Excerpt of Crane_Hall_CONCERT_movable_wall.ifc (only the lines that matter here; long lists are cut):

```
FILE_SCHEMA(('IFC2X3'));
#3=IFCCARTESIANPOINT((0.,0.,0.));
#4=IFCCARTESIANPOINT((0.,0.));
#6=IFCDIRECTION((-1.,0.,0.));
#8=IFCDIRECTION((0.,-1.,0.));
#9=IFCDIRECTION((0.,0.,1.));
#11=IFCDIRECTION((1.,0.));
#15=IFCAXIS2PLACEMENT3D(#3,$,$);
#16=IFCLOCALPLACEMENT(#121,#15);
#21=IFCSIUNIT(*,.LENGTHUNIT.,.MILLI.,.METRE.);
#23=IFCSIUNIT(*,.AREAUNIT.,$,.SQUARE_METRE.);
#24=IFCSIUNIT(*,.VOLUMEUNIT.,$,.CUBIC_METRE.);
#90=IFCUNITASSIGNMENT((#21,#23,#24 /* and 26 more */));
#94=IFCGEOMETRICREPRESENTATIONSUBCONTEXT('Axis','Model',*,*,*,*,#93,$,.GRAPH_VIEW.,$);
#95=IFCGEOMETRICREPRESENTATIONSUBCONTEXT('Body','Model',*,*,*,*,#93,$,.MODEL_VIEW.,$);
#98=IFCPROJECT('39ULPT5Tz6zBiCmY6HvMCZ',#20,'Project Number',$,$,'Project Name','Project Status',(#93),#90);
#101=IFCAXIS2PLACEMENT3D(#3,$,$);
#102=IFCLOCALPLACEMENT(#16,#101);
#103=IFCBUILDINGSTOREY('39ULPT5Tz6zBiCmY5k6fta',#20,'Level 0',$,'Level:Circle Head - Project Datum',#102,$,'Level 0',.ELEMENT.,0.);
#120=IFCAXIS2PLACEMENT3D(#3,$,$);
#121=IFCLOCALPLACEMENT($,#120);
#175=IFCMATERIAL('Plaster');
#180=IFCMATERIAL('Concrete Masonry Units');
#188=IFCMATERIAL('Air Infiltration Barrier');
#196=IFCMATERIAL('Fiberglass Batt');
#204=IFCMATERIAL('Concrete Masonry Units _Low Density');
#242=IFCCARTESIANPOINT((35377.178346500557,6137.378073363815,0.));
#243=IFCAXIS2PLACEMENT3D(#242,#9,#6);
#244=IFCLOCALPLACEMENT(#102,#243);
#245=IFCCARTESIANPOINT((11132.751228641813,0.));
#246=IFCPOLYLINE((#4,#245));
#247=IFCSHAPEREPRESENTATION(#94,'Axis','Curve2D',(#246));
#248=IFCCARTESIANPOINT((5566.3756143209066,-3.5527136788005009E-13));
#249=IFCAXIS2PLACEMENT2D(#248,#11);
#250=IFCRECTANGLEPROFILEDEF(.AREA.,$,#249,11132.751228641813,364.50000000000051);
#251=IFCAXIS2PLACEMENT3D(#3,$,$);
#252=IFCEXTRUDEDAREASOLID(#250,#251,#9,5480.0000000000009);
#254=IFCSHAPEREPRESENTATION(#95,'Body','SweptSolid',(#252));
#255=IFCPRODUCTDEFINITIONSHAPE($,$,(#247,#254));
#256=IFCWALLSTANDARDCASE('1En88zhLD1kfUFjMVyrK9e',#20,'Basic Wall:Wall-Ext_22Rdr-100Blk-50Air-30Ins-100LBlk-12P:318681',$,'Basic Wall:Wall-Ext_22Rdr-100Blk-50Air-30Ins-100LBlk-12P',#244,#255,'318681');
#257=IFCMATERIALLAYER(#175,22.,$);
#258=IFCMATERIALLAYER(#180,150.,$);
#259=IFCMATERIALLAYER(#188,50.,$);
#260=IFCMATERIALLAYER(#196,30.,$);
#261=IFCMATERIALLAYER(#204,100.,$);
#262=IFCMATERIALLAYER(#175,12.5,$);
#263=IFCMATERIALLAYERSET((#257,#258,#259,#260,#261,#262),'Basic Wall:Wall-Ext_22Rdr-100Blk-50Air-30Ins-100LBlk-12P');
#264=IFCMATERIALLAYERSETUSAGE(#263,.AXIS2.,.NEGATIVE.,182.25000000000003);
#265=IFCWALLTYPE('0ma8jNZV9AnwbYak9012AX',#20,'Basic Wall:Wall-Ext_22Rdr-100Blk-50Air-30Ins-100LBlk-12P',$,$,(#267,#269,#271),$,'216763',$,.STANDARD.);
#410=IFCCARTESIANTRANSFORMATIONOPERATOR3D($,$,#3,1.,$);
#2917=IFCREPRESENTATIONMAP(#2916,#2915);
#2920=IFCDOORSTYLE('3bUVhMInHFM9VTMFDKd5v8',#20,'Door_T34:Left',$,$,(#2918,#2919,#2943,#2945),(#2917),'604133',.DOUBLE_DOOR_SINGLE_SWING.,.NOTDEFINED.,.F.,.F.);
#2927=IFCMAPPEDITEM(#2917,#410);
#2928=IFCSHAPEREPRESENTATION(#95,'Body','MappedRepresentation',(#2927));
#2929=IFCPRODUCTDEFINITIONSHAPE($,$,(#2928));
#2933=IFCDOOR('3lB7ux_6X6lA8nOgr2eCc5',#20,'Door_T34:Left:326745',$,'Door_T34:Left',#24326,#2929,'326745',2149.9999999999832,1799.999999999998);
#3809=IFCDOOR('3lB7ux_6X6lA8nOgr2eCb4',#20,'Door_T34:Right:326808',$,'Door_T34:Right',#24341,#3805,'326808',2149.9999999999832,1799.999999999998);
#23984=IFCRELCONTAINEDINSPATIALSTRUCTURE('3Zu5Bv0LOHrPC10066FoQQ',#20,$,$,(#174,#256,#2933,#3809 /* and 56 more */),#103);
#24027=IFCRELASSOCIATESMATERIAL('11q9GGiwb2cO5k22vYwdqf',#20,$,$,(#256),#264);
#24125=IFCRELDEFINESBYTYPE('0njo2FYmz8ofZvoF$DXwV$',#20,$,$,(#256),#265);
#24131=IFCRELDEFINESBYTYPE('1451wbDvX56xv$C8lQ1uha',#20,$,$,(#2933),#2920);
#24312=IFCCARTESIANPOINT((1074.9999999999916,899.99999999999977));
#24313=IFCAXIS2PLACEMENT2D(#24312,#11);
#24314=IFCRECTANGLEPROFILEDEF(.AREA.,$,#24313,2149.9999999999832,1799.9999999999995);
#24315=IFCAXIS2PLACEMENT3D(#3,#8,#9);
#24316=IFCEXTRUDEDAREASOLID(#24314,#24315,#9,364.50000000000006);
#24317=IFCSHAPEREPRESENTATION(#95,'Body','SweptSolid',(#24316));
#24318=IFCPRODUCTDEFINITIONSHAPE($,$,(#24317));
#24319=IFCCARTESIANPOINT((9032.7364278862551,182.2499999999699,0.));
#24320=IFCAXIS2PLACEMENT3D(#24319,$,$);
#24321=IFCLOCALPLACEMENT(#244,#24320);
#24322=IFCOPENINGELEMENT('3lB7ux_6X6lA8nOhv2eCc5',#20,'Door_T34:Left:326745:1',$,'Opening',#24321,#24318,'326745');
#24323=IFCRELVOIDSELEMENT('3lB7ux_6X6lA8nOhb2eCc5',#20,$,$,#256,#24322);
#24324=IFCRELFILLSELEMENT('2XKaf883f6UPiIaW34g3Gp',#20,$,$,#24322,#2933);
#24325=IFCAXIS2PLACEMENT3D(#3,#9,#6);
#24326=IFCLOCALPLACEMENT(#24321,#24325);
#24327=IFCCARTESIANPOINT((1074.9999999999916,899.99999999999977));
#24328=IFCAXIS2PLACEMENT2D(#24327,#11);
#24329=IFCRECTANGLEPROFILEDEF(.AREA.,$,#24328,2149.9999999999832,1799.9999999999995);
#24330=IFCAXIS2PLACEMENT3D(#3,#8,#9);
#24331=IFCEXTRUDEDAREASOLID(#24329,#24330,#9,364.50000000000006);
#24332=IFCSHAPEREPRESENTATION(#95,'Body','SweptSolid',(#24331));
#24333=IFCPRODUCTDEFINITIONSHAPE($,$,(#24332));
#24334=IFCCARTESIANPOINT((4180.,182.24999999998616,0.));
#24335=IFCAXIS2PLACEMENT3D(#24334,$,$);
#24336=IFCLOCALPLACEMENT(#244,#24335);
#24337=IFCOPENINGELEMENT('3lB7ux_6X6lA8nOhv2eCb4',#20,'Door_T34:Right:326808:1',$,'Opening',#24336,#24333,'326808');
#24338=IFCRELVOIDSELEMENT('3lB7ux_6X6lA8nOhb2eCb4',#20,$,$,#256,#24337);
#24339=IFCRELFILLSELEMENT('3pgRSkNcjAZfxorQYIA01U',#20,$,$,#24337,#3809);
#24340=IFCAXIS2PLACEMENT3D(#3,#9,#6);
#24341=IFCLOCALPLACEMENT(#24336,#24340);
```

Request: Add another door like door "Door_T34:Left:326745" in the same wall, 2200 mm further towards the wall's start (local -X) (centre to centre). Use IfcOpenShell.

```python
import ifcopenshell
import ifcopenshell.api.feature
import ifcopenshell.api.geometry
import ifcopenshell.api.root
import ifcopenshell.geom
import ifcopenshell.util.element
import ifcopenshell.util.placement
import ifcopenshell.util.shape

model = ifcopenshell.open("Crane_Hall_CONCERT_movable_wall.ifc")
settings = ifcopenshell.geom.settings()


def volume(element):
    """Net volume in cubic metres, openings subtracted."""
    shape = ifcopenshell.geom.create_shape(settings, element)
    return ifcopenshell.util.shape.get_volume(shape.geometry)


def reuse_history(source, copy):
    """copy_class also copies each property set's owner history, people and application; keep the originals."""
    for rel in copy.IsDefinedBy:
        if rel.is_a("IfcRelDefinesByProperties") and (history := rel.RelatingPropertyDefinition.OwnerHistory):
            rel.RelatingPropertyDefinition.OwnerHistory = source.OwnerHistory
            ifcopenshell.util.element.remove_deep2(model, history)


door = model.by_guid("3lB7ux_6X6lA8nOgr2eCc5")
opening = door.FillsVoids[0].RelatingOpeningElement
wall = opening.VoidsElements[0].RelatingBuildingElement
before = volume(wall)
shift = ifcopenshell.util.placement.get_local_placement(wall.ObjectPlacement)[:3, 0] * -2200.0

# copy_class copies the void relationship, type, container and properties, but no geometry.
new_opening = ifcopenshell.api.root.copy_class(model, product=opening)
new_opening.Representation = ifcopenshell.util.element.copy_deep(
    model, opening.Representation, exclude=["IfcGeometricRepresentationContext", "IfcRepresentationMap"]
)
new_opening.Name = "Door_T34:Left"
new_opening.Tag = None
new_door = ifcopenshell.api.root.copy_class(model, product=door)
new_door.Representation = ifcopenshell.util.element.copy_deep(
    model, door.Representation, exclude=["IfcGeometricRepresentationContext", "IfcRepresentationMap"]
)
new_door.Name = "Door_T34:Left"
new_door.Tag = None
reuse_history(door, new_door)
fills = ifcopenshell.api.feature.add_filling(model, opening=new_opening, element=new_door)
fills.OwnerHistory = new_door.OwnerHistory  # required in IFC2X3

for old, new in ((opening, new_opening), (door, new_door)):
    matrix = ifcopenshell.util.placement.get_local_placement(old.ObjectPlacement)
    matrix[:3, 3] += shift
    ifcopenshell.api.geometry.edit_object_placement(model, product=new, matrix=matrix, is_si=False)

after = volume(wall)

print(f"wall volume {before:.3f} -> {after:.3f} m3")

model.write("Crane_Hall_CONCERT_movable_wall_v2.ifc")
```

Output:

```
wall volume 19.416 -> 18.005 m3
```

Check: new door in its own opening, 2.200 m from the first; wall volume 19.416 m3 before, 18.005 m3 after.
